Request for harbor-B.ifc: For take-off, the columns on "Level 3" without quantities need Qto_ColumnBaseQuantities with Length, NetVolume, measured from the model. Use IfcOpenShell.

First a look at what the model holds.

```python
import ifcopenshell
import ifcopenshell.util.element
import ifcopenshell.util.unit

model = ifcopenshell.open("harbor-B.ifc")
print(model.schema)
for unit_type in ("LENGTHUNIT", "AREAUNIT", "VOLUMEUNIT"):
    print(unit_type, ifcopenshell.util.unit.calculate_unit_scale(model, unit_type))
storey = next(s for s in model.by_type("IfcBuildingStorey") if s.Name == "Level 3")
columns = [e for e in ifcopenshell.util.element.get_decomposition(storey) if e.is_a("IfcColumn")]
for e in sorted(columns, key=lambda e: e.id()):
    print(e.id(), e.is_a(), e.Name, list(ifcopenshell.util.element.get_psets(e, qtos_only=True)), sep=" | ")
```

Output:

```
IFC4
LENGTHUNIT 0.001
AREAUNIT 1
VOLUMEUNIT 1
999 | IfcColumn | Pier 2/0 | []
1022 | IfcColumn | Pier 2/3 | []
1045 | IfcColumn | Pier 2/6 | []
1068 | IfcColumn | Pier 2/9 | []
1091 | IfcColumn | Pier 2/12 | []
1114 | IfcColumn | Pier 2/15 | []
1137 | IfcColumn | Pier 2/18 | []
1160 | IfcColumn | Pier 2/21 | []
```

```python
import ifcopenshell
import ifcopenshell.api.pset
import ifcopenshell.geom
import ifcopenshell.util.element
import ifcopenshell.util.shape
import ifcopenshell.util.unit

model = ifcopenshell.open("harbor-B.ifc")
unit_scale = ifcopenshell.util.unit.calculate_unit_scale(model)
volume_scale = ifcopenshell.util.unit.calculate_unit_scale(model, "VOLUMEUNIT")
settings = ifcopenshell.geom.settings()

storey = next(s for s in model.by_type("IfcBuildingStorey") if s.Name == "Level 3")
columns = [e for e in ifcopenshell.util.element.get_decomposition(storey) if e.is_a("IfcColumn")]

for e in sorted(columns, key=lambda e: e.id()):
    if ifcopenshell.util.element.get_psets(e, qtos_only=True, should_inherit=False):
        continue
    # Geometry comes back in metres, in the element's own axes.
    shape = ifcopenshell.geom.create_shape(settings, e)
    values = {
        "Length": ifcopenshell.util.shape.get_z(shape.geometry) / unit_scale,
        "NetVolume": ifcopenshell.util.shape.get_volume(shape.geometry) / volume_scale,
    }
    qto = ifcopenshell.api.pset.add_qto(model, product=e, name="Qto_ColumnBaseQuantities")
    ifcopenshell.api.pset.edit_qto(model, qto=qto, properties=values)
    print(e.id(), {k: round(v, 3) for k, v in values.items()})

model.write("harbor-B_v2.ifc")
```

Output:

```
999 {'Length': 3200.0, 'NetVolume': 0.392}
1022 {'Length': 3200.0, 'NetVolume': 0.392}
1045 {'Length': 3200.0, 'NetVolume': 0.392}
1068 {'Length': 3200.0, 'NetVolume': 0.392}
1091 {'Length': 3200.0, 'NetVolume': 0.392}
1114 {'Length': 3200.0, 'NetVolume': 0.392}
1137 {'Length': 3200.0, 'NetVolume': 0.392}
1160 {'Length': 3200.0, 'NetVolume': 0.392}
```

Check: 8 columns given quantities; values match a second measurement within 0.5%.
